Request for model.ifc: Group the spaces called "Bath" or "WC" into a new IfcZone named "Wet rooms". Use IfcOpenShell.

First a look at what the model holds.

```python
import ifcopenshell

model = ifcopenshell.open("model.ifc")
print(model.schema)
seen = {}
for space in model.by_type("IfcSpace"):
    seen[space.LongName] = seen.get(space.LongName, 0) + 1
for name, count in sorted(seen.items(), key=str):
    print(count, "x", name)
print("zones:", [z.Name for z in model.by_type("IfcZone")][:20])
```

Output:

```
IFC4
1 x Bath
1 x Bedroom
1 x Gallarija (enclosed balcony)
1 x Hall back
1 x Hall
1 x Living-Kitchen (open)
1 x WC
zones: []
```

```python
import ifcopenshell
import ifcopenshell.api.group
import ifcopenshell.api.root

model = ifcopenshell.open("model.ifc")

names = {"Bath", "WC"}
spaces = [s for s in model.by_type("IfcSpace") if s.LongName in names]

zone = ifcopenshell.api.root.create_entity(model, ifc_class="IfcZone", name="Wet rooms")
ifcopenshell.api.group.assign_group(model, products=spaces, group=zone)
print(len(spaces), "spaces in", zone.Name)

model.write("model_edited.ifc")
```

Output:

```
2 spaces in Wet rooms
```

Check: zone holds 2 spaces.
